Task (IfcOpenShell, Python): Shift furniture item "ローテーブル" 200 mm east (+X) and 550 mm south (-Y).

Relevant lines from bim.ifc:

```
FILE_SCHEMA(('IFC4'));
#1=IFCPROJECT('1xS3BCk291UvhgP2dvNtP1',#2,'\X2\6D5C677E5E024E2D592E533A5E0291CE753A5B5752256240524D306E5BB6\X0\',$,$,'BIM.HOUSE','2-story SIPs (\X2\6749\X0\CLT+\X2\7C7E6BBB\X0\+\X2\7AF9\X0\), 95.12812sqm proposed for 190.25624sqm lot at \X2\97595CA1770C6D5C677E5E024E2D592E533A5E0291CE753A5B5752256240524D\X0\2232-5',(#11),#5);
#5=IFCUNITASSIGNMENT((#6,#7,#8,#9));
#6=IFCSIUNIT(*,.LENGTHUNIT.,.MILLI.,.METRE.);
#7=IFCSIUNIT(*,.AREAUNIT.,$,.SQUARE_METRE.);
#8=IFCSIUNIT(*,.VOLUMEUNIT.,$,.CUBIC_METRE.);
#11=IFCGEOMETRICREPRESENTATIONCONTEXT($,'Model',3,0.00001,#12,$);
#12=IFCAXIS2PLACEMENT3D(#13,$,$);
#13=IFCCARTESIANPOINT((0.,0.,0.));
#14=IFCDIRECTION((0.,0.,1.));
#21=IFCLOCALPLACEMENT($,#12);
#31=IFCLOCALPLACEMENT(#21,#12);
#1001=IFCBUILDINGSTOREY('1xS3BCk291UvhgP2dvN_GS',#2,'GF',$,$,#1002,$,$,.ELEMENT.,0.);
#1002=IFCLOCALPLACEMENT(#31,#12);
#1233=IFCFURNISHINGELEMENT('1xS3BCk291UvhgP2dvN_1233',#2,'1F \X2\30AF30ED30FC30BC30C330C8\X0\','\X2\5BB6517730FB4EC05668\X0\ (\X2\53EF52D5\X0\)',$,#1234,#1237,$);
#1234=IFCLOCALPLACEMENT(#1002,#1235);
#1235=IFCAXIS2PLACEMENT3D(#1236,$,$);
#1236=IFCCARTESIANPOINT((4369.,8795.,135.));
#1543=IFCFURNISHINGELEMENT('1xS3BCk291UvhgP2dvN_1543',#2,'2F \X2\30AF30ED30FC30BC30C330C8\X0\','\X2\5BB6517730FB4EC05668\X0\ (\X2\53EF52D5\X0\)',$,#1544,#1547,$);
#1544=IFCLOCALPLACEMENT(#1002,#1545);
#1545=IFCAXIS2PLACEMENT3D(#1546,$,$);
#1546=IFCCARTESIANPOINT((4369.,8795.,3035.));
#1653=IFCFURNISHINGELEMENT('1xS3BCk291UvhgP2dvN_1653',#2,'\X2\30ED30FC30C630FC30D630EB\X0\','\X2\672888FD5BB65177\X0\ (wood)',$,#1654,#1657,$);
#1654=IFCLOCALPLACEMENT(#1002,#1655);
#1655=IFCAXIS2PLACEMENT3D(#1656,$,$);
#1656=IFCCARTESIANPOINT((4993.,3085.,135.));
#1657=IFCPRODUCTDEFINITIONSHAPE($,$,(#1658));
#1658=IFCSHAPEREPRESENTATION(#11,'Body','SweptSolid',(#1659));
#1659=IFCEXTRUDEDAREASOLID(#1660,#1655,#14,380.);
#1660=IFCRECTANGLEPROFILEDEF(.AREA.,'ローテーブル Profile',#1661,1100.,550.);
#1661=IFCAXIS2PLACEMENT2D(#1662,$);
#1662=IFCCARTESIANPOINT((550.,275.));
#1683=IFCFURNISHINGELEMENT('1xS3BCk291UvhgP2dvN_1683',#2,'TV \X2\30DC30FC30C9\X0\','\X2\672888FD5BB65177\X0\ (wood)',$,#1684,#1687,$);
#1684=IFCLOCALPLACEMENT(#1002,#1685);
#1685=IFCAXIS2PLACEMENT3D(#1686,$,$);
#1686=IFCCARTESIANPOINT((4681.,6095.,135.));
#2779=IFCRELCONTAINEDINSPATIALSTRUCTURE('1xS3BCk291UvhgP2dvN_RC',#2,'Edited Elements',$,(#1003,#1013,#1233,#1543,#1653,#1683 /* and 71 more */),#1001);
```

```python
import ifcopenshell
import ifcopenshell.api.geometry
import ifcopenshell.util.placement

model = ifcopenshell.open("bim.ifc")

item = model.by_guid("1xS3BCk291UvhgP2dvN_1653")
matrix = ifcopenshell.util.placement.get_local_placement(item.ObjectPlacement)
matrix[0, 3] += 200.0
matrix[1, 3] -= 550.0
ifcopenshell.api.geometry.edit_object_placement(model, product=item, matrix=matrix, is_si=False)

print(ifcopenshell.util.placement.get_local_placement(item.ObjectPlacement).round(3) + 0.0)

model.write("bim_rev.ifc")
```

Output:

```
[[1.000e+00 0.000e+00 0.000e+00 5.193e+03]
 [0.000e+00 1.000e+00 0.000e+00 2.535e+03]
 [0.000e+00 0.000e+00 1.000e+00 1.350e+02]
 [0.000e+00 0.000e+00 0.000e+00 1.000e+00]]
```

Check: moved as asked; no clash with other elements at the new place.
